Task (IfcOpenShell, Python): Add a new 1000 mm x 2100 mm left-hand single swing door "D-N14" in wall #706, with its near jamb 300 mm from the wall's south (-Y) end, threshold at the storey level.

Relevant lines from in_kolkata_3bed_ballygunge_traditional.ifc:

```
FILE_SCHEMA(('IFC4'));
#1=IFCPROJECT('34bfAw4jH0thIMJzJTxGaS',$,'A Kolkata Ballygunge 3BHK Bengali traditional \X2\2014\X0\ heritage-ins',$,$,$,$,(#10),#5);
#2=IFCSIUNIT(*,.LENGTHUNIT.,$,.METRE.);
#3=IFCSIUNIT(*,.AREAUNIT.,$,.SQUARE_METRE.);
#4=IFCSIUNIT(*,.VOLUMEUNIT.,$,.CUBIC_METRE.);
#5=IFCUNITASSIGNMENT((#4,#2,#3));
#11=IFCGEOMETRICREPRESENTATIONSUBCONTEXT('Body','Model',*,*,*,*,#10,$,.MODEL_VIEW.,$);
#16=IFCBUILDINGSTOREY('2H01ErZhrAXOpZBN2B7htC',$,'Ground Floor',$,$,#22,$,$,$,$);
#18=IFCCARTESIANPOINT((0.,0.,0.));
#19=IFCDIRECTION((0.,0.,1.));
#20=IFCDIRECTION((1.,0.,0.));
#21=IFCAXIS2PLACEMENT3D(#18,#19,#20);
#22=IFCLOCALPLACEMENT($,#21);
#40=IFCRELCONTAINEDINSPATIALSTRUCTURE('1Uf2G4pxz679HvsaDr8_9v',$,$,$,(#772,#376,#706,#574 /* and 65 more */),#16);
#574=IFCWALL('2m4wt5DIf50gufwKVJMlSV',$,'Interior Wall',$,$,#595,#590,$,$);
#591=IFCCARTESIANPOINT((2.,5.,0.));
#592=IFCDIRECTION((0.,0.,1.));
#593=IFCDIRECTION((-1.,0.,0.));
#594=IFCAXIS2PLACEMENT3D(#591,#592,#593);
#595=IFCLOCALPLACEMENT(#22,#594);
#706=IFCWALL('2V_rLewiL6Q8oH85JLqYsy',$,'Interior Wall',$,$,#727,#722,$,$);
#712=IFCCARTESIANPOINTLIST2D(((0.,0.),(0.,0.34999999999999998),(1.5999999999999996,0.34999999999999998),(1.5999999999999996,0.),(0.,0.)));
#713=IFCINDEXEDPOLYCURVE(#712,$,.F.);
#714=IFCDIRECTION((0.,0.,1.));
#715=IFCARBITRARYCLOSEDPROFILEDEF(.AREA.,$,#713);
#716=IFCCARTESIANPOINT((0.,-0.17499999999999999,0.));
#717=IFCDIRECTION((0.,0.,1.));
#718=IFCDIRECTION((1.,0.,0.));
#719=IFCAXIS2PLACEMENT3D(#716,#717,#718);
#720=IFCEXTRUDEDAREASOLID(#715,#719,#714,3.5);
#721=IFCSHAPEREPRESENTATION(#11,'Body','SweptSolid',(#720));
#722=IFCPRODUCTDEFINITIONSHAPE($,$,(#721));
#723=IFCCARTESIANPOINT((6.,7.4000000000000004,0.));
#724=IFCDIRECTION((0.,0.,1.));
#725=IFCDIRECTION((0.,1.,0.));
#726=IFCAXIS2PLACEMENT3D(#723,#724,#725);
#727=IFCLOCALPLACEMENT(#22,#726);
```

```python
import numpy as np
import ifcopenshell
import ifcopenshell.api.feature
import ifcopenshell.api.geometry
import ifcopenshell.api.root
import ifcopenshell.api.spatial
import ifcopenshell.geom
import ifcopenshell.util.element
import ifcopenshell.util.placement
import ifcopenshell.util.representation
import ifcopenshell.util.shape
import ifcopenshell.util.unit

model = ifcopenshell.open("in_kolkata_3bed_ballygunge_traditional.ifc")
unit_scale = ifcopenshell.util.unit.calculate_unit_scale(model)
settings = ifcopenshell.geom.settings()


def volume(element):
    """Net volume in cubic metres, openings subtracted."""
    shape = ifcopenshell.geom.create_shape(settings, element)
    return ifcopenshell.util.shape.get_volume(shape.geometry)


wall = model.by_guid("2V_rLewiL6Q8oH85JLqYsy")
storey = ifcopenshell.util.element.get_container(wall, ifc_class="IfcBuildingStorey")
context = ifcopenshell.util.representation.get_context(model, "Model", "Body", "MODEL_VIEW")
before = volume(wall)

width, height, from_end, sill = 1, 2.1, 0.3, 0.0  # metres

# The wall runs along its own X axis, and the end named is its -X end.
wall_shape = ifcopenshell.geom.create_shape(settings, wall)
x, y, z = ifcopenshell.util.shape.get_vertices(wall_shape.geometry).T
start = x.min() + from_end
face, thickness = float(y.min()), float(y.max() - y.min())
wall_matrix = ifcopenshell.util.placement.get_local_placement(wall.ObjectPlacement)
level = ifcopenshell.util.placement.get_local_placement(storey.ObjectPlacement)[2, 3]


def in_wall(x, y):
    """Placement at x, y metres in the wall's axes, at sill height."""
    matrix = wall_matrix.copy()
    matrix[:, 3] = wall_matrix @ np.array([x / unit_scale, y / unit_scale, 0.0, 1.0])
    matrix[2, 3] = level + sill / unit_scale
    return matrix


# Opening: a box that overshoots both wall faces by 50 mm.
opening = ifcopenshell.api.root.create_entity(model, ifc_class="IfcOpeningElement", predefined_type="OPENING")
box = ifcopenshell.api.geometry.add_wall_representation(
    model, context=context, length=width, height=height, thickness=thickness + 0.1
)
ifcopenshell.api.geometry.assign_representation(model, product=opening, representation=box)
ifcopenshell.api.geometry.edit_object_placement(model, product=opening, matrix=in_wall(start, face - 0.05), is_si=False)
ifcopenshell.api.feature.add_feature(model, feature=opening, element=wall)

door = ifcopenshell.api.root.create_entity(model, ifc_class="IfcDoor", name="D-N14", predefined_type="DOOR")
door.OverallWidth, door.OverallHeight = width / unit_scale, height / unit_scale
door.OperationType = "SINGLE_SWING_LEFT"
body = ifcopenshell.api.geometry.add_door_representation(
    model,
    context=context,
    overall_width=door.OverallWidth,
    overall_height=door.OverallHeight,
    operation_type="SINGLE_SWING_LEFT",
    lining_properties={"LiningDepth": thickness / unit_scale, "ThresholdDepth": thickness / unit_scale},
)
ifcopenshell.api.geometry.assign_representation(model, product=door, representation=body)
ifcopenshell.api.spatial.assign_container(model, products=[door], relating_structure=storey)
ifcopenshell.api.feature.add_filling(model, opening=opening, element=door)

# The lining spans the wall, so the door starts at the wall face.
ifcopenshell.api.geometry.edit_object_placement(model, product=door, matrix=in_wall(start, face), is_si=False)

after = volume(wall)

print(f"wall volume {before:.3f} -> {after:.3f} m3")

model.write("in_kolkata_3bed_ballygunge_traditional_edited.ifc")
```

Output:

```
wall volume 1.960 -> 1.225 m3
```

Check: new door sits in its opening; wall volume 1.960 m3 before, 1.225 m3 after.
